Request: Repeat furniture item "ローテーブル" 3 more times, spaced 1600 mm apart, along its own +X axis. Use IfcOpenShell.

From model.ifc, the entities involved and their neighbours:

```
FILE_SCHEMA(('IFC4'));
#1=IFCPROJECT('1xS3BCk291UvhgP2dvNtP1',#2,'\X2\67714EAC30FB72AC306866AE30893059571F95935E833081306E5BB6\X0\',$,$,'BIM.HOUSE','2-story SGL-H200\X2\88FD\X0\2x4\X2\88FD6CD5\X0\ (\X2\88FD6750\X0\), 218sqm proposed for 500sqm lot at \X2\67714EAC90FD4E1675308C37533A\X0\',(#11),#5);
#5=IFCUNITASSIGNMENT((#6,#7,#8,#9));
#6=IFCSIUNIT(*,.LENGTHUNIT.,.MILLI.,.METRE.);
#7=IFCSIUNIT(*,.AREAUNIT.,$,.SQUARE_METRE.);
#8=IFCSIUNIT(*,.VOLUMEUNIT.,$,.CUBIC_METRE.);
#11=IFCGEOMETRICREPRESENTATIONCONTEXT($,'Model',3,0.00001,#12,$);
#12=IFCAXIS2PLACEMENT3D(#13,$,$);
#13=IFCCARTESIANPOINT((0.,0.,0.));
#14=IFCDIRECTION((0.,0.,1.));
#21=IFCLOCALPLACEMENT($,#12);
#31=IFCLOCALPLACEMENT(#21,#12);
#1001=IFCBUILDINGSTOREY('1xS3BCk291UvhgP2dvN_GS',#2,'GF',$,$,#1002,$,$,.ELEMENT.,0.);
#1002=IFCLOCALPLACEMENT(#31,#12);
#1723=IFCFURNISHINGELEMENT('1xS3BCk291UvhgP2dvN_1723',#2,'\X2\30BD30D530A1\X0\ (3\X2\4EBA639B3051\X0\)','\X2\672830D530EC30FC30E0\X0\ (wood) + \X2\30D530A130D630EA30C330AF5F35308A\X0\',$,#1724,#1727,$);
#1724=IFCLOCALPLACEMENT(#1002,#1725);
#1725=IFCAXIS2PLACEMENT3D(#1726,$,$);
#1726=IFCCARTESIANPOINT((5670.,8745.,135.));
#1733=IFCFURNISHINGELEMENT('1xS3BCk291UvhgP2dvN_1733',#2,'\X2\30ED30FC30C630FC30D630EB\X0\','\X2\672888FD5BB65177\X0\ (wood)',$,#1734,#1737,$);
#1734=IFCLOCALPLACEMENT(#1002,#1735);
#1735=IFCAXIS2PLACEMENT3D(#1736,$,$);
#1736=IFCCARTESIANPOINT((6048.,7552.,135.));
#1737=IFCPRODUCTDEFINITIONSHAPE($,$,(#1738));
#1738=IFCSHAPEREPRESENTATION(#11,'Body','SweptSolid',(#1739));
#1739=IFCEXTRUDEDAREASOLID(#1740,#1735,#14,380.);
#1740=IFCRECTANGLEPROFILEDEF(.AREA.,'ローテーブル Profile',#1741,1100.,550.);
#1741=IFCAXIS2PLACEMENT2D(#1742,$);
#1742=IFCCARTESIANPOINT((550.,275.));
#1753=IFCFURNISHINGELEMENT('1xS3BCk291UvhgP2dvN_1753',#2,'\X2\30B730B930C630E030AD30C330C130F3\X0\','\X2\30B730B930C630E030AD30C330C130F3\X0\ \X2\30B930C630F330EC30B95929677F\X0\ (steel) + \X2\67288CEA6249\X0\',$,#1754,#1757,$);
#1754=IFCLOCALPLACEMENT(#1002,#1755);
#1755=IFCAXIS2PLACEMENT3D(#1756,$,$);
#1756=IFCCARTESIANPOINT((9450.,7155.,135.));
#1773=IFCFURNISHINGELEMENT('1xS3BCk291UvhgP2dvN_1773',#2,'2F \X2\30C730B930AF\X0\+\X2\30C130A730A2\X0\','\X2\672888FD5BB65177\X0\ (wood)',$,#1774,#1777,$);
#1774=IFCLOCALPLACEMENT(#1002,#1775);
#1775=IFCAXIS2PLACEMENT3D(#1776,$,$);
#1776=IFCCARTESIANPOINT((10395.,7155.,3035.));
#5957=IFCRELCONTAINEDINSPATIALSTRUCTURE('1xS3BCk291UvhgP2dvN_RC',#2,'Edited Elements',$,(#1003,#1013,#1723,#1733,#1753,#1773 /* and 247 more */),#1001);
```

```python
import ifcopenshell
import ifcopenshell.api.geometry
import ifcopenshell.api.root
import ifcopenshell.util.element
import ifcopenshell.util.placement
import ifcopenshell.util.unit

model = ifcopenshell.open("model.ifc")
unit_scale = ifcopenshell.util.unit.calculate_unit_scale(model)


def reuse_history(source, copy):
    """copy_class also copies each property set's owner history, people and application; keep the originals."""
    for rel in copy.IsDefinedBy:
        if rel.is_a("IfcRelDefinesByProperties") and (history := rel.RelatingPropertyDefinition.OwnerHistory):
            rel.RelatingPropertyDefinition.OwnerHistory = source.OwnerHistory
            ifcopenshell.util.element.remove_deep2(model, history)


source = model.by_id(1733)
base = ifcopenshell.util.placement.get_local_placement(source.ObjectPlacement)
step = base[:3, 0] * 1.6 / unit_scale

for i in range(1, 4):
    copy = ifcopenshell.api.root.copy_class(model, product=source)
    copy.Representation = ifcopenshell.util.element.copy_deep(
        model, source.Representation, exclude=["IfcGeometricRepresentationContext", "IfcRepresentationMap"]
    )
    reuse_history(source, copy)
    matrix = base.copy()
    matrix[:3, 3] += i * step
    print("added at", matrix[:3, 3].round(3) + 0.0)
    ifcopenshell.api.geometry.edit_object_placement(model, product=copy, matrix=matrix, is_si=False)

model.write("model_edited.ifc")
```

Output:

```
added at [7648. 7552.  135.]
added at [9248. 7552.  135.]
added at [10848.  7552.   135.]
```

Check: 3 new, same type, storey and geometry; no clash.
